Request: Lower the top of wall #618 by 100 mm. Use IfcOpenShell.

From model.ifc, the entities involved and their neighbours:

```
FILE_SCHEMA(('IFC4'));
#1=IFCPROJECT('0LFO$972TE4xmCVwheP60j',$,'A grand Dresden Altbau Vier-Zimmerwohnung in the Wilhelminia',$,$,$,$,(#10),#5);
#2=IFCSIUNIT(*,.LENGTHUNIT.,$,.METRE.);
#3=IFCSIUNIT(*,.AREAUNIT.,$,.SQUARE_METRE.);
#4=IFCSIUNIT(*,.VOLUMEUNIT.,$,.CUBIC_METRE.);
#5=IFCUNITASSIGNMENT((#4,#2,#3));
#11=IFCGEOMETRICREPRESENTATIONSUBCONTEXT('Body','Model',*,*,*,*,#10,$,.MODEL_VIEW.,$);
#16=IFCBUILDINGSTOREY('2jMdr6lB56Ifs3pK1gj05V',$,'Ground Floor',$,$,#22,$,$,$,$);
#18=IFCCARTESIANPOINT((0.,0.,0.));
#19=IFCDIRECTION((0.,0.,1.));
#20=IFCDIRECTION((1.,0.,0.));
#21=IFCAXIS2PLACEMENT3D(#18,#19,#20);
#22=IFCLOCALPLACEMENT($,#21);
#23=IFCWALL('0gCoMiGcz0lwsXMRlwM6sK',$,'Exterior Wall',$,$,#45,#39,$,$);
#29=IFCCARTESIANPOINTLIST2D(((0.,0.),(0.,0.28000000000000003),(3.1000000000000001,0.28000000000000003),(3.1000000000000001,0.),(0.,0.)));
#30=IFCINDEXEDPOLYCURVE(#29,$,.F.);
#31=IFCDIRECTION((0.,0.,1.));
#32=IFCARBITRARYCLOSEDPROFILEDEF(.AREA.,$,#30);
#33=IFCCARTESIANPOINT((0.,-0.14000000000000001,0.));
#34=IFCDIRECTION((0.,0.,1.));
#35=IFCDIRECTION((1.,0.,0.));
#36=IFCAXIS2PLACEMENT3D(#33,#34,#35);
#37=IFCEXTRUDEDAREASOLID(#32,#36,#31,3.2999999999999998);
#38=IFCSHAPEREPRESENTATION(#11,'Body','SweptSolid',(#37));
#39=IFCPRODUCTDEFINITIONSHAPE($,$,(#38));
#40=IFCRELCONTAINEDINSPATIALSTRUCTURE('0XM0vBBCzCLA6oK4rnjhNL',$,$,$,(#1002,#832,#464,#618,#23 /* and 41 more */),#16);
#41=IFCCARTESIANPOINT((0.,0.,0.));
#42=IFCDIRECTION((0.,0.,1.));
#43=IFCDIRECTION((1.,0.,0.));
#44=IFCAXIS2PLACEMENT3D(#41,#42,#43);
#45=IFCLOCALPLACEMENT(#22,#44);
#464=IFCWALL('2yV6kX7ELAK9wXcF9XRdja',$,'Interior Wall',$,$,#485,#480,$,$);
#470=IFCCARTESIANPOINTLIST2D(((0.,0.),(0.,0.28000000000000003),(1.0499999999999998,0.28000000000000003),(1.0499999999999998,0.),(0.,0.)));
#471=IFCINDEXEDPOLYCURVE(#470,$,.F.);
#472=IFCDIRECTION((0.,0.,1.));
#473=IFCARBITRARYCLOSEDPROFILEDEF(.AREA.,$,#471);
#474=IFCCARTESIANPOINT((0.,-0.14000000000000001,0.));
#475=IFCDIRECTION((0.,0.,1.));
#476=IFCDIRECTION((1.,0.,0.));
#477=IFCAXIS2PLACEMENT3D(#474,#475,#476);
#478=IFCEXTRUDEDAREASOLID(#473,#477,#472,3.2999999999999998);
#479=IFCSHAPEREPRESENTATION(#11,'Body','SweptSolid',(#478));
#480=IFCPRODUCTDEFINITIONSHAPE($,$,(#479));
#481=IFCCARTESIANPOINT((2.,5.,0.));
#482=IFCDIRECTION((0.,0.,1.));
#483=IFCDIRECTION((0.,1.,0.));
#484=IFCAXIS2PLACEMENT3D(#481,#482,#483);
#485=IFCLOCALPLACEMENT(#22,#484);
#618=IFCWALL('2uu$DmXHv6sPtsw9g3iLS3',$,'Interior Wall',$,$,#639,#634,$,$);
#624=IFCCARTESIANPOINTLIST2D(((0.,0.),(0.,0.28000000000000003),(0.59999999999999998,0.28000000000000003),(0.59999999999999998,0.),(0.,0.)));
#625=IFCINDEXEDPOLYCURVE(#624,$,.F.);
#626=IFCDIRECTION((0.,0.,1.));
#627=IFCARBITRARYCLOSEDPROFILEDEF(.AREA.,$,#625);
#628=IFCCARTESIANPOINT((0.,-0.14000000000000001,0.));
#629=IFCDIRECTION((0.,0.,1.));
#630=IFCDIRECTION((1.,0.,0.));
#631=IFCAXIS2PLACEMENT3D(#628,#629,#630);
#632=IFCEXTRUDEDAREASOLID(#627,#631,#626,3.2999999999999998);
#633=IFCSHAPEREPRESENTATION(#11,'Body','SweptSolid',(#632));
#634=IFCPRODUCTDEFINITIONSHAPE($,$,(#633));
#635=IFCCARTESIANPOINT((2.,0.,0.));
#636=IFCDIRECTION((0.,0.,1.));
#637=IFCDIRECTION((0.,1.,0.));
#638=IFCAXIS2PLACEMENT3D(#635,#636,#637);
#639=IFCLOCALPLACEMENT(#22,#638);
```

```python
import ifcopenshell
import ifcopenshell.geom
import ifcopenshell.util.representation
import ifcopenshell.util.shape

model = ifcopenshell.open("model.ifc")
settings = ifcopenshell.geom.settings()


def volume(element):
    """Net volume in cubic metres, openings subtracted."""
    shape = ifcopenshell.geom.create_shape(settings, element)
    return ifcopenshell.util.shape.get_volume(shape.geometry)


wall = model.by_id(618)
before = volume(wall)

body = ifcopenshell.util.representation.get_representation(wall, "Model", "Body")
solid = body.Items[0]
old_height = solid.Depth
solid.Depth -= 0.1
after = volume(wall)

print(f"height {old_height:g} -> {solid.Depth:g}, volume {before:.3f} -> {after:.3f} m3")

model.write("model_updated.ifc")
```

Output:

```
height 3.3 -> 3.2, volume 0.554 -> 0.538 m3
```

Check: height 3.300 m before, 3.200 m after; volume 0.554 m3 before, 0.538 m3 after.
